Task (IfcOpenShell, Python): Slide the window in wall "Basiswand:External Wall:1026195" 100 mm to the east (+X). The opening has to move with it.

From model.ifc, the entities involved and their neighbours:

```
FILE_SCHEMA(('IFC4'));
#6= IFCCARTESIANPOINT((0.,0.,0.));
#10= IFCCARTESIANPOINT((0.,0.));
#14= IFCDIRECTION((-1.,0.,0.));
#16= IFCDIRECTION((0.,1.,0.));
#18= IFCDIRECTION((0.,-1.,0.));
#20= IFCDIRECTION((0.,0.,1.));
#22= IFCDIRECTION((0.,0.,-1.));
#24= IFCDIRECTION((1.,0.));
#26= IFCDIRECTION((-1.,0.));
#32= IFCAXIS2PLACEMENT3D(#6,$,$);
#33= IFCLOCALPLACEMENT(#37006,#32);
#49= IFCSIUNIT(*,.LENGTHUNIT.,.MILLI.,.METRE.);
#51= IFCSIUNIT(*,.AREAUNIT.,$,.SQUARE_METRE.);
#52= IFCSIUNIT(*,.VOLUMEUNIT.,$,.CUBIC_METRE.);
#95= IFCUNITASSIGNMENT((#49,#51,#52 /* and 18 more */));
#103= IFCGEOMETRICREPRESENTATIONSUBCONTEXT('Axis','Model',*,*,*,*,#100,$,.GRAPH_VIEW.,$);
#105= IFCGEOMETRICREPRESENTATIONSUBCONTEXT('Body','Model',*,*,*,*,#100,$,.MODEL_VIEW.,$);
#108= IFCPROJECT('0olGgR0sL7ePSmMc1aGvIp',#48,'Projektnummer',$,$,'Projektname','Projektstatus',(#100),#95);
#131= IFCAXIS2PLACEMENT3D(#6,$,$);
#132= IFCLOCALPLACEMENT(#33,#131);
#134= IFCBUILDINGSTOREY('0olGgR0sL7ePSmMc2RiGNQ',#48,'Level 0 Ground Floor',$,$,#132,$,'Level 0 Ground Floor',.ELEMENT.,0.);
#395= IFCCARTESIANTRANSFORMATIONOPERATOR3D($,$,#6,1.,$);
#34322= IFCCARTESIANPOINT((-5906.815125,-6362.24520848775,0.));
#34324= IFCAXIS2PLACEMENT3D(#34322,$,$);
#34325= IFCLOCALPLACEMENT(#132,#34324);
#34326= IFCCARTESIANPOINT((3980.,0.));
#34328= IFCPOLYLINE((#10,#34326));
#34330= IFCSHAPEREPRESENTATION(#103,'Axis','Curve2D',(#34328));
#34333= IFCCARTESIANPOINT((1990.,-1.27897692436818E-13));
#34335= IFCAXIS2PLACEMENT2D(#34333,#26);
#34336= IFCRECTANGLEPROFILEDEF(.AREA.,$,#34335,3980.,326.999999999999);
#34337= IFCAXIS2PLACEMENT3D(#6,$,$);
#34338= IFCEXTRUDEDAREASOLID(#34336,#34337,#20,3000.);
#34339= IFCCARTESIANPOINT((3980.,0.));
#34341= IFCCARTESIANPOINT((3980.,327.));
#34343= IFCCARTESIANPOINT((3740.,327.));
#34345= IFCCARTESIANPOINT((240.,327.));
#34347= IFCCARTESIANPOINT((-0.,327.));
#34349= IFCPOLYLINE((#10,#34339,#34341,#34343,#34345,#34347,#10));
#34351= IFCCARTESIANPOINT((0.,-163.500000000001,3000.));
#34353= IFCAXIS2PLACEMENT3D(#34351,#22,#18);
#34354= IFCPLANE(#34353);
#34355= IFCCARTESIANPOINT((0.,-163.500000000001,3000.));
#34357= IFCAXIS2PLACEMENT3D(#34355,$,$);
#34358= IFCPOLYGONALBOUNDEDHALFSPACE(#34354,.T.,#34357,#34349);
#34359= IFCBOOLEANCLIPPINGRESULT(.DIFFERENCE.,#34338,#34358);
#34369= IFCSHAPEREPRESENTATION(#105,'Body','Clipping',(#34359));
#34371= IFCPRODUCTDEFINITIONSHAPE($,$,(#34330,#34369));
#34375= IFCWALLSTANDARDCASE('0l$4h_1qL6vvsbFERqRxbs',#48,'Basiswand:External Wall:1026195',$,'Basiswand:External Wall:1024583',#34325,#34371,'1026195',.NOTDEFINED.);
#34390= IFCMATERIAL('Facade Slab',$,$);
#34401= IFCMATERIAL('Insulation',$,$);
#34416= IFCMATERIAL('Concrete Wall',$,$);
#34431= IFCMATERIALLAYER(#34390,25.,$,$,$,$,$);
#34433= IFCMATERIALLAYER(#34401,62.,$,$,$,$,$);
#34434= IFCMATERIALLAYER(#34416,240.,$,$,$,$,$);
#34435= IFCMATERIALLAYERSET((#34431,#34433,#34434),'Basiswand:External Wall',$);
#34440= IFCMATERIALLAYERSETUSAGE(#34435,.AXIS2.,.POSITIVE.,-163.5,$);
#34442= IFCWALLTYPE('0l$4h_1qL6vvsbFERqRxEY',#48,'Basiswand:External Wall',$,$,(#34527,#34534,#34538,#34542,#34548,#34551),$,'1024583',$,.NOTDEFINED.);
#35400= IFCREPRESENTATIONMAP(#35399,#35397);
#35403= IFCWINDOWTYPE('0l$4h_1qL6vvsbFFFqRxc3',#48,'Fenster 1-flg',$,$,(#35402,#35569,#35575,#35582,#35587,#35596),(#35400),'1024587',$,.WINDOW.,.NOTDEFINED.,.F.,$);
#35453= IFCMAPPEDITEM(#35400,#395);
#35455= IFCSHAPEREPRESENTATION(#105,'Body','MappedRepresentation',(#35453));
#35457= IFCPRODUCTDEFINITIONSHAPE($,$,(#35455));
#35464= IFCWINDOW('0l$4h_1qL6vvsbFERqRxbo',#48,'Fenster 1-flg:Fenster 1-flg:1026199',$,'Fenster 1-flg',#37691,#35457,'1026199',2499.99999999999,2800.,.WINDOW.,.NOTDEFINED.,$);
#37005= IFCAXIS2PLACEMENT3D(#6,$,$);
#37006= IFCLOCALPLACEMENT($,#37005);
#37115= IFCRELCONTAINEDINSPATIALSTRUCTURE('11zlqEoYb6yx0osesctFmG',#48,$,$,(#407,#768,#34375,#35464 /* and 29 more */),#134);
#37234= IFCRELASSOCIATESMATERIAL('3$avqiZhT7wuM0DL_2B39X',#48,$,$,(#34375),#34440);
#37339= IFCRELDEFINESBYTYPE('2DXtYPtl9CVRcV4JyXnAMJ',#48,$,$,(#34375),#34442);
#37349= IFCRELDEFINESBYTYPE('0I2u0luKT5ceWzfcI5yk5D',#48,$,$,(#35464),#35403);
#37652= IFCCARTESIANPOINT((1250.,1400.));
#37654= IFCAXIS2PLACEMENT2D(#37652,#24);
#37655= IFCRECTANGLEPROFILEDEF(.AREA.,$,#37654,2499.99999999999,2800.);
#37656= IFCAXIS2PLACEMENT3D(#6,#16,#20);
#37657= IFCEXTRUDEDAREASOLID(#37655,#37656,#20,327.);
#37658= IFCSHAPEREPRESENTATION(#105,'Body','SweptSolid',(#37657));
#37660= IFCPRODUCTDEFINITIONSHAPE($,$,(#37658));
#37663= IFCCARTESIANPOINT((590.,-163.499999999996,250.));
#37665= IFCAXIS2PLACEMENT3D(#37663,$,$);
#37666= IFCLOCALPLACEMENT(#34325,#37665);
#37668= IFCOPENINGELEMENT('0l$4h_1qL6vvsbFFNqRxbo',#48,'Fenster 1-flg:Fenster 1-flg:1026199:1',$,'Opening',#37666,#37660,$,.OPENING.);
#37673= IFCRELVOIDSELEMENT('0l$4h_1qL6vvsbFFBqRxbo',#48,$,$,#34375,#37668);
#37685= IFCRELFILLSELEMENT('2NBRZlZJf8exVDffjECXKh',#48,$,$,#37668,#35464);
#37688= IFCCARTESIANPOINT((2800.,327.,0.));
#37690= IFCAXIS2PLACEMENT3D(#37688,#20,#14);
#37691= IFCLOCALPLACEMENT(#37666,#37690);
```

```python
import ifcopenshell
import ifcopenshell.api.geometry
import ifcopenshell.util.placement
import ifcopenshell.util.unit

model = ifcopenshell.open("model.ifc")
unit_scale = ifcopenshell.util.unit.calculate_unit_scale(model)

window = model.by_guid("0l$4h_1qL6vvsbFERqRxbo")
opening = window.FillsVoids[0].RelatingOpeningElement
wall = opening.VoidsElements[0].RelatingBuildingElement

wall_matrix = ifcopenshell.util.placement.get_local_placement(wall.ObjectPlacement)
shift = wall_matrix[:3, 0] * 0.1 / unit_scale
before = ifcopenshell.util.placement.get_local_placement(window.ObjectPlacement)[:3, 3].copy()

# The window is placed relative to its opening, so it follows when the opening moves.
matrix = ifcopenshell.util.placement.get_local_placement(opening.ObjectPlacement)
matrix[:3, 3] += shift
ifcopenshell.api.geometry.edit_object_placement(
    model, product=opening, matrix=matrix, is_si=False, should_transform_children=True
)

after = ifcopenshell.util.placement.get_local_placement(window.ObjectPlacement)[:3, 3]
print("window moved by", (after - before).round(3) + 0.0)

model.write("model_updated.ifc")
```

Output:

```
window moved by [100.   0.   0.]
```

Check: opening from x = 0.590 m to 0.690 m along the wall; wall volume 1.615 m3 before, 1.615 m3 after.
